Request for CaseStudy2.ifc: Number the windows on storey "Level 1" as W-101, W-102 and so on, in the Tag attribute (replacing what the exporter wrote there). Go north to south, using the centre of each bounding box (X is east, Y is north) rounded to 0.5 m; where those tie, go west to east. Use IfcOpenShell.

First a look at what the model holds.

```python
import ifcopenshell
import ifcopenshell.util.element
import ifcopenshell.util.placement

model = ifcopenshell.open("CaseStudy2.ifc")
print(model.schema)
storey = next(s for s in model.by_type("IfcBuildingStorey") if s.Name == "Level 1")
windows = [e for e in ifcopenshell.util.element.get_decomposition(storey) if e.is_a("IfcWindow")]
for e in sorted(windows, key=lambda e: e.id()):
    origin = ifcopenshell.util.placement.get_local_placement(e.ObjectPlacement)[:3, 3]
    print(e.id(), e.Tag, e.Name, origin.round(2) + 0.0, sep=" | ")
```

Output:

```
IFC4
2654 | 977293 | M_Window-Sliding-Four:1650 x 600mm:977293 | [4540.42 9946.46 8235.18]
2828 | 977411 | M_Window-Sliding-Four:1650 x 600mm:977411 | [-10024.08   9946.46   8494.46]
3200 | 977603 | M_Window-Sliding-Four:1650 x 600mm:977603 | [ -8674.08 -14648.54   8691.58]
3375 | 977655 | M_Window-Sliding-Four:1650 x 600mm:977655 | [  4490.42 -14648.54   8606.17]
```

```python
import ifcopenshell
import ifcopenshell.geom
import ifcopenshell.util.element
import ifcopenshell.util.shape

model = ifcopenshell.open("CaseStudy2.ifc")
settings = ifcopenshell.geom.settings()
settings.set("use-world-coords", True)


def centre(element):
    shape = ifcopenshell.geom.create_shape(settings, element)
    return ifcopenshell.util.shape.get_bbox_centroid(shape.geometry)


storey = next(s for s in model.by_type("IfcBuildingStorey") if s.Name == "Level 1")
windows = [e for e in ifcopenshell.util.element.get_decomposition(storey) if e.is_a("IfcWindow")]

# Insertion points can sit at a corner or the storey origin, so sort by the geometry (in metres).
centres = {e: centre(e) for e in windows}
windows.sort(key=lambda e: (-round(centres[e][1] / 0.5), centres[e][0]))

for i, e in enumerate(windows, start=1):
    number = f"W-1{i:02d}"
    e.Tag = number
    print(e.id(), number)

model.write("CaseStudy2_rev.ifc")
```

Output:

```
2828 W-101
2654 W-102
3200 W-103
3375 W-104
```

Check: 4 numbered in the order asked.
